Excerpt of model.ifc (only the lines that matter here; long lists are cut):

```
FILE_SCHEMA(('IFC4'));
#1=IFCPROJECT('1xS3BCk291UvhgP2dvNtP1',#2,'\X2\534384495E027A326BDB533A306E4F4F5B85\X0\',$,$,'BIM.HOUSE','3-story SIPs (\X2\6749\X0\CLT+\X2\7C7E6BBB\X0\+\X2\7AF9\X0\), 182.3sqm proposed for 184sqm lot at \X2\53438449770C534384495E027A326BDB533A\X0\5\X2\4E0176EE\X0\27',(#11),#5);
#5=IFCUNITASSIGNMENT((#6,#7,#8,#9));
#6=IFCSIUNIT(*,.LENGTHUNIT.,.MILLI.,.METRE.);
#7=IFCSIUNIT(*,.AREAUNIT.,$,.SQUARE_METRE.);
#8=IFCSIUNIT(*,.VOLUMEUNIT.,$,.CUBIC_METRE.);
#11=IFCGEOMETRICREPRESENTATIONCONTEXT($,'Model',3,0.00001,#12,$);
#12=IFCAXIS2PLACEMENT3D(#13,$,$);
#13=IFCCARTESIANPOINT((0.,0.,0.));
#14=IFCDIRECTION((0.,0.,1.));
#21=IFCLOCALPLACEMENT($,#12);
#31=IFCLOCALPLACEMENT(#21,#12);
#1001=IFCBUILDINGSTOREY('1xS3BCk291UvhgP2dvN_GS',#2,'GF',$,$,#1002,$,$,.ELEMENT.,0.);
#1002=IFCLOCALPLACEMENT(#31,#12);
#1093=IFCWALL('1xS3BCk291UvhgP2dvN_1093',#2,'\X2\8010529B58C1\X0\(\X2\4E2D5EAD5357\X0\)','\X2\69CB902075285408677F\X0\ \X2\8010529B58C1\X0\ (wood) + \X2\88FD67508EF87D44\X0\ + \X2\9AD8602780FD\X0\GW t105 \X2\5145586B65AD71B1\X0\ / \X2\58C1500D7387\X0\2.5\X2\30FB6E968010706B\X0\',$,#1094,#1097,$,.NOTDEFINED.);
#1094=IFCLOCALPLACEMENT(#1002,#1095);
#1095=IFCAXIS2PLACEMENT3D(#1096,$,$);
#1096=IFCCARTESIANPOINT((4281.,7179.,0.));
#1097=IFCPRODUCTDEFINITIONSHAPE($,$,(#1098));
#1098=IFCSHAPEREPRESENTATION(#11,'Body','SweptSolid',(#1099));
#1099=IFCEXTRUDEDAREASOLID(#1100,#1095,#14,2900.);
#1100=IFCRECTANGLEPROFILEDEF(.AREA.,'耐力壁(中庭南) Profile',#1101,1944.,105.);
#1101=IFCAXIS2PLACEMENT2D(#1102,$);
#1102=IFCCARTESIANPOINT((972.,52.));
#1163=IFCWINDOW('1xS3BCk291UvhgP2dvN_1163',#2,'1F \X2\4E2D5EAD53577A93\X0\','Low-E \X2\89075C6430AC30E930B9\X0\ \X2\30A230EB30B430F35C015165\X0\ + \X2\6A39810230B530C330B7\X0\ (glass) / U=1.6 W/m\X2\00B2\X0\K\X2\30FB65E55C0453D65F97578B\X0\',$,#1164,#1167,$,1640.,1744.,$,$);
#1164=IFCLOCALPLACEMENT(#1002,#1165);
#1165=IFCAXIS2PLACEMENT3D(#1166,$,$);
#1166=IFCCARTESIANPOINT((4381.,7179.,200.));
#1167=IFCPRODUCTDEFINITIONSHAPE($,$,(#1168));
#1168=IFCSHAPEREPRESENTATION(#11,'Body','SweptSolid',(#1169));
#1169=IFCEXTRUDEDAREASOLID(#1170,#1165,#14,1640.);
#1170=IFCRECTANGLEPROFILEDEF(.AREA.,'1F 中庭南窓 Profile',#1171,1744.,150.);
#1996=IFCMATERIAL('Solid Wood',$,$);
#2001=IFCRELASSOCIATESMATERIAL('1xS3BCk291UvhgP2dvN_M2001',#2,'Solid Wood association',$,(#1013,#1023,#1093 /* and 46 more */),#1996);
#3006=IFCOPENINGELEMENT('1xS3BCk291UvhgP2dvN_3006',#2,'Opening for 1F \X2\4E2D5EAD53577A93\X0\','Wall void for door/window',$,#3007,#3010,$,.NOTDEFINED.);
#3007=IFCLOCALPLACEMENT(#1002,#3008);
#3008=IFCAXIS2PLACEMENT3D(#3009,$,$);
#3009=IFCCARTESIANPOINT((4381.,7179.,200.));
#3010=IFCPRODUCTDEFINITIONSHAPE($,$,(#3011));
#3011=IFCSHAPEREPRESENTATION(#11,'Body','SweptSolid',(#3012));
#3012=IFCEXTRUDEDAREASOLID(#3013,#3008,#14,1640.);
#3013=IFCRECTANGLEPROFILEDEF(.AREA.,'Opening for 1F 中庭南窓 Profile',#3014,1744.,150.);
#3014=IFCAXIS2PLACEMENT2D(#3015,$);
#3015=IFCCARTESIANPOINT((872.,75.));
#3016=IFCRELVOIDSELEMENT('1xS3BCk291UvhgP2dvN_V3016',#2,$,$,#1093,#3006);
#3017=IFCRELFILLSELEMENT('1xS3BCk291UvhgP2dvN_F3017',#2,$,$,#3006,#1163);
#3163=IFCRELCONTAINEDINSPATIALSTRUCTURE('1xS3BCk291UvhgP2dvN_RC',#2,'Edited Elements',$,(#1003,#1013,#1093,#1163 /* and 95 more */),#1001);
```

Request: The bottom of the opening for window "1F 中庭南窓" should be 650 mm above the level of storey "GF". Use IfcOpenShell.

```python
import numpy as np
import ifcopenshell
import ifcopenshell.api.geometry
import ifcopenshell.geom
import ifcopenshell.util.element
import ifcopenshell.util.placement
import ifcopenshell.util.shape
import ifcopenshell.util.unit

model = ifcopenshell.open("model.ifc")
unit_scale = ifcopenshell.util.unit.calculate_unit_scale(model)

window = model.by_guid("1xS3BCk291UvhgP2dvN_1163")
opening = window.FillsVoids[0].RelatingOpeningElement
storey = ifcopenshell.util.element.get_container(window, ifc_class="IfcBuildingStorey")
level = ifcopenshell.util.placement.get_local_placement(storey.ObjectPlacement)[2, 3]

# The opening's origin need not be at the sill, so measure its lowest point.
shape = ifcopenshell.geom.create_shape(ifcopenshell.geom.settings(), opening)
bottom = ifcopenshell.util.shape.get_shape_bottom_elevation(shape, shape.geometry) / unit_scale
dz = level + 0.65 / unit_scale - bottom

shift = np.array([0.0, 0.0, dz])
# The window is not placed relative to its opening, so move both.
for product in (opening, window):
    matrix = ifcopenshell.util.placement.get_local_placement(product.ObjectPlacement)
    matrix[:3, 3] += shift
    ifcopenshell.api.geometry.edit_object_placement(model, product=product, matrix=matrix, is_si=False)

print(f"moved by {dz * unit_scale:+.3f} m")

model.write("model_rev.ifc")
```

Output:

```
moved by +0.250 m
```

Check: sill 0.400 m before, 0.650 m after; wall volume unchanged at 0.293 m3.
